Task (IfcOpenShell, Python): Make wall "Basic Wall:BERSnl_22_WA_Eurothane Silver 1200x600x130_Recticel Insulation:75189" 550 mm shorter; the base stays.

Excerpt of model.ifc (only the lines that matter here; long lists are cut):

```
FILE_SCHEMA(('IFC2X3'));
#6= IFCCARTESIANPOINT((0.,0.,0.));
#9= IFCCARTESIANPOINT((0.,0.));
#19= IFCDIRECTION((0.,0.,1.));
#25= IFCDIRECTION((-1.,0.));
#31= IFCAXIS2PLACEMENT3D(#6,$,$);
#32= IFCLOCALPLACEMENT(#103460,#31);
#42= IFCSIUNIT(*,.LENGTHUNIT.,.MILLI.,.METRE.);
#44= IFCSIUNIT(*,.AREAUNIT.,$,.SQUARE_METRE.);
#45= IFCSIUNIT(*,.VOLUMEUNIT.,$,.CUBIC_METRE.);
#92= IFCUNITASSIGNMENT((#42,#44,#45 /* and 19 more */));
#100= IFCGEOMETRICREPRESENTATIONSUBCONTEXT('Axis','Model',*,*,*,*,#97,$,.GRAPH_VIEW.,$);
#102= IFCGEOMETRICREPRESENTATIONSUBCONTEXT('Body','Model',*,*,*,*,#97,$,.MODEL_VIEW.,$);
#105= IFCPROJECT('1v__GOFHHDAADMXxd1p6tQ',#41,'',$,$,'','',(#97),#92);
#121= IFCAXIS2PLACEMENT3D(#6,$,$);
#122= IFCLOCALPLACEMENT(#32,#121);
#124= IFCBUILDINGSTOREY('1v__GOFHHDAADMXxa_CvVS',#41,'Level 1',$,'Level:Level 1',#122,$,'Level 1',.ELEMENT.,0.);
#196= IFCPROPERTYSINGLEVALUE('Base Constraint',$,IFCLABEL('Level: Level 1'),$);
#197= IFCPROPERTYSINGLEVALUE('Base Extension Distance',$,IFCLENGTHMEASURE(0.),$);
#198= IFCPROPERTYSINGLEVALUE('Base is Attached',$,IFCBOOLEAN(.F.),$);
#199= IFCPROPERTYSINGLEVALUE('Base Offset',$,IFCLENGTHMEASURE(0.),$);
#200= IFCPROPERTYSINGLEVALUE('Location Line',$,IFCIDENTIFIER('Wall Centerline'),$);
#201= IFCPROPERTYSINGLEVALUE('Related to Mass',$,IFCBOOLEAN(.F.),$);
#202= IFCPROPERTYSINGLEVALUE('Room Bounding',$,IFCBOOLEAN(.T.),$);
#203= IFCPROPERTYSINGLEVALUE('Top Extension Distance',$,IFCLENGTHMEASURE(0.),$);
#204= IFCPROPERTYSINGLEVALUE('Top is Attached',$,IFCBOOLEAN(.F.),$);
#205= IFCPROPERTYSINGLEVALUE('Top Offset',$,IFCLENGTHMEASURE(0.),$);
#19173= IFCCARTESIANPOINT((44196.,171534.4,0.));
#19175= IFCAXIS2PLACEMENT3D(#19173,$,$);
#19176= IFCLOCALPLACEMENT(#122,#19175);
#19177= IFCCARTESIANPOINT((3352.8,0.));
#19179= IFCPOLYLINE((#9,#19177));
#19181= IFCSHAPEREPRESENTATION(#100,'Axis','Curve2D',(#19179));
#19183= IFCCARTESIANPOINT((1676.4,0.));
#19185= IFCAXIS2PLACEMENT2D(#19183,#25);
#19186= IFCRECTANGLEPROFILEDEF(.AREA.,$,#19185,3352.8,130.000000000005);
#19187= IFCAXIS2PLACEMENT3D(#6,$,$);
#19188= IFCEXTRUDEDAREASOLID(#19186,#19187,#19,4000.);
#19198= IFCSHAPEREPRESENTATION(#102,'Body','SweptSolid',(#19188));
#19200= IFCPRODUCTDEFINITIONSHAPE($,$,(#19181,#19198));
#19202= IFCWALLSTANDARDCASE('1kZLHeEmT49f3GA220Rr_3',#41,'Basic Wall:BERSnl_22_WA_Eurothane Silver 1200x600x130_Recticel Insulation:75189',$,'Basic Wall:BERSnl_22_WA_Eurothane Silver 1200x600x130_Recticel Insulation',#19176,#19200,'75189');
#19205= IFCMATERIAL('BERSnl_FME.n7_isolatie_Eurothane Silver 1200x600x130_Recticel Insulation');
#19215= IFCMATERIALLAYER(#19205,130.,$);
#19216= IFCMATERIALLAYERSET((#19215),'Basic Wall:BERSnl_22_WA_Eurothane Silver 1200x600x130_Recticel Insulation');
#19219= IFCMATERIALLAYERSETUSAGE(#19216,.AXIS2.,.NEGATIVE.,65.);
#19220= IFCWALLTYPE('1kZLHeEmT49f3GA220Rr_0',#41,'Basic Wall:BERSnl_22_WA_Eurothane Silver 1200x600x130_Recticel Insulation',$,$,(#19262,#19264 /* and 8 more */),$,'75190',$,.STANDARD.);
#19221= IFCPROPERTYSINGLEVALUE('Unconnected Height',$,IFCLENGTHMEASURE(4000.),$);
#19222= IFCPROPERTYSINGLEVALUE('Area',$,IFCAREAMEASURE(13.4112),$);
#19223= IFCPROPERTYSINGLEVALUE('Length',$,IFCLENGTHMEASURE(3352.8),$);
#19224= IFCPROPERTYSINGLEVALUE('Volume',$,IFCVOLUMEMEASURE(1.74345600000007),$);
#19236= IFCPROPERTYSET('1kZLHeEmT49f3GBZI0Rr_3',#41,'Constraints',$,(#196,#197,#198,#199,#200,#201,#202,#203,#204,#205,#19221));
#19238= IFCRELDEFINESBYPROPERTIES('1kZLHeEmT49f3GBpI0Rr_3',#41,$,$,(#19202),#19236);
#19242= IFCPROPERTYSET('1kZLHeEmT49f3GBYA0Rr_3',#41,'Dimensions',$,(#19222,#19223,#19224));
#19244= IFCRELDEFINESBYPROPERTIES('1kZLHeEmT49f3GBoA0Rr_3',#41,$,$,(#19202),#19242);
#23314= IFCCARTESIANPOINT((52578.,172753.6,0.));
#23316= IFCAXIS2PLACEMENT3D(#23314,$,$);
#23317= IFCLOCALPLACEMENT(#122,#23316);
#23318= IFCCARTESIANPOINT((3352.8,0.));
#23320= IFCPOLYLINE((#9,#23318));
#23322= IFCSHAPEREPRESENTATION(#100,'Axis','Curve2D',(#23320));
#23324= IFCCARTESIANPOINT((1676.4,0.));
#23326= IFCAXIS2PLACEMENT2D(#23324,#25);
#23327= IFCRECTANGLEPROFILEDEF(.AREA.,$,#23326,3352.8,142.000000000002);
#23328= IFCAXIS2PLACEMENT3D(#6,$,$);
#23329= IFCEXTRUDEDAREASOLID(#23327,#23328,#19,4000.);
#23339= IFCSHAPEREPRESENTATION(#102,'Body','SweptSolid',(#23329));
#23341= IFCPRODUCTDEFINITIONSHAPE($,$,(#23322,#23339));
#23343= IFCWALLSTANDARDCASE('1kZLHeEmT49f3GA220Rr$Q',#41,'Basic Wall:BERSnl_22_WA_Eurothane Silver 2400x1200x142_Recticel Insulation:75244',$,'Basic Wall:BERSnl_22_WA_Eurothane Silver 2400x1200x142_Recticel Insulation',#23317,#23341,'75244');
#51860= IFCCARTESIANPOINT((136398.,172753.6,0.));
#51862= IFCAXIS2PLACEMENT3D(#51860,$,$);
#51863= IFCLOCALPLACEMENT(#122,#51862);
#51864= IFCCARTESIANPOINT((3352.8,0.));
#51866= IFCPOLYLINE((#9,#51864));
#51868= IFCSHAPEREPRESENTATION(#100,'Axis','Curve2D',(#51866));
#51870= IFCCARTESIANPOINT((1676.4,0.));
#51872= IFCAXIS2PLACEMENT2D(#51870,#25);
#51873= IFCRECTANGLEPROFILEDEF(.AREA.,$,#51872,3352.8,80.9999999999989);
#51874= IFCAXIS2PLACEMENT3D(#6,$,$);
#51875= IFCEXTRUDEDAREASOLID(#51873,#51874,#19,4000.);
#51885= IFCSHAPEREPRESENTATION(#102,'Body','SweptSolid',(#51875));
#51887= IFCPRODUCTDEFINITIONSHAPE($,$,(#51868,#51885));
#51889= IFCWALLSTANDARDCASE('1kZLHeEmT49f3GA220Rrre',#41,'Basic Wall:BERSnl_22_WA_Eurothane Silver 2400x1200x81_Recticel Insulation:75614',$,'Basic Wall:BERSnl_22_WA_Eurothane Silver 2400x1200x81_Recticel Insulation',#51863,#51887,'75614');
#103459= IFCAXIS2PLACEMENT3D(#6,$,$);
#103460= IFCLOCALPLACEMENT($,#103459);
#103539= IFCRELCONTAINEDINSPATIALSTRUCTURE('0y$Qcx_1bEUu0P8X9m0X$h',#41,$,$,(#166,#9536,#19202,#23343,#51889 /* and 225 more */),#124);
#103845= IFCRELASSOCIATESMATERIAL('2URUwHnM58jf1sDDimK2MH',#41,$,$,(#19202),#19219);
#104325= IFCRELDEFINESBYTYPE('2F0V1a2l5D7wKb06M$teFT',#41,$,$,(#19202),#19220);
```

```python
import ifcopenshell
import ifcopenshell.api.pset
import ifcopenshell.geom
import ifcopenshell.util.element
import ifcopenshell.util.representation
import ifcopenshell.util.shape
import ifcopenshell.util.unit

model = ifcopenshell.open("model.ifc")
unit_scale = ifcopenshell.util.unit.calculate_unit_scale(model)
area_scale = ifcopenshell.util.unit.calculate_unit_scale(model, "AREAUNIT")
volume_scale = ifcopenshell.util.unit.calculate_unit_scale(model, "VOLUMEUNIT")
settings = ifcopenshell.geom.settings()


def volume(element):
    """Net volume in cubic metres, openings subtracted."""
    shape = ifcopenshell.geom.create_shape(settings, element)
    return ifcopenshell.util.shape.get_volume(shape.geometry)


wall = model.by_id(19202)
before = volume(wall)

body = ifcopenshell.util.representation.get_representation(wall, "Model", "Body")
solid = body.Items[0]
old_height = solid.Depth
solid.Depth -= 0.55 / unit_scale
after = volume(wall)
thickness = 0.13  # wall thickness in metres

# Update the stored height, areas and volumes.
pset = model.by_id(ifcopenshell.util.element.get_pset(wall, "Constraints", should_inherit=False)["id"])
ifcopenshell.api.pset.edit_pset(model, pset=pset, properties={
    "Unconnected Height": model.create_entity("IfcLengthMeasure", solid.Depth),
})
pset = model.by_id(ifcopenshell.util.element.get_pset(wall, "Dimensions", should_inherit=False)["id"])
ifcopenshell.api.pset.edit_pset(model, pset=pset, properties={
    "Area": model.create_entity("IfcAreaMeasure", after / thickness / area_scale),
    "Volume": model.create_entity("IfcVolumeMeasure", after / volume_scale),
})

print(f"height {old_height:g} -> {solid.Depth:g}, volume {before:.3f} -> {after:.3f} m3")

model.write("model_updated.ifc")
```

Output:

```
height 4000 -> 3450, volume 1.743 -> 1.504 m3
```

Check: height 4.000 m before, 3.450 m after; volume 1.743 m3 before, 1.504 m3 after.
